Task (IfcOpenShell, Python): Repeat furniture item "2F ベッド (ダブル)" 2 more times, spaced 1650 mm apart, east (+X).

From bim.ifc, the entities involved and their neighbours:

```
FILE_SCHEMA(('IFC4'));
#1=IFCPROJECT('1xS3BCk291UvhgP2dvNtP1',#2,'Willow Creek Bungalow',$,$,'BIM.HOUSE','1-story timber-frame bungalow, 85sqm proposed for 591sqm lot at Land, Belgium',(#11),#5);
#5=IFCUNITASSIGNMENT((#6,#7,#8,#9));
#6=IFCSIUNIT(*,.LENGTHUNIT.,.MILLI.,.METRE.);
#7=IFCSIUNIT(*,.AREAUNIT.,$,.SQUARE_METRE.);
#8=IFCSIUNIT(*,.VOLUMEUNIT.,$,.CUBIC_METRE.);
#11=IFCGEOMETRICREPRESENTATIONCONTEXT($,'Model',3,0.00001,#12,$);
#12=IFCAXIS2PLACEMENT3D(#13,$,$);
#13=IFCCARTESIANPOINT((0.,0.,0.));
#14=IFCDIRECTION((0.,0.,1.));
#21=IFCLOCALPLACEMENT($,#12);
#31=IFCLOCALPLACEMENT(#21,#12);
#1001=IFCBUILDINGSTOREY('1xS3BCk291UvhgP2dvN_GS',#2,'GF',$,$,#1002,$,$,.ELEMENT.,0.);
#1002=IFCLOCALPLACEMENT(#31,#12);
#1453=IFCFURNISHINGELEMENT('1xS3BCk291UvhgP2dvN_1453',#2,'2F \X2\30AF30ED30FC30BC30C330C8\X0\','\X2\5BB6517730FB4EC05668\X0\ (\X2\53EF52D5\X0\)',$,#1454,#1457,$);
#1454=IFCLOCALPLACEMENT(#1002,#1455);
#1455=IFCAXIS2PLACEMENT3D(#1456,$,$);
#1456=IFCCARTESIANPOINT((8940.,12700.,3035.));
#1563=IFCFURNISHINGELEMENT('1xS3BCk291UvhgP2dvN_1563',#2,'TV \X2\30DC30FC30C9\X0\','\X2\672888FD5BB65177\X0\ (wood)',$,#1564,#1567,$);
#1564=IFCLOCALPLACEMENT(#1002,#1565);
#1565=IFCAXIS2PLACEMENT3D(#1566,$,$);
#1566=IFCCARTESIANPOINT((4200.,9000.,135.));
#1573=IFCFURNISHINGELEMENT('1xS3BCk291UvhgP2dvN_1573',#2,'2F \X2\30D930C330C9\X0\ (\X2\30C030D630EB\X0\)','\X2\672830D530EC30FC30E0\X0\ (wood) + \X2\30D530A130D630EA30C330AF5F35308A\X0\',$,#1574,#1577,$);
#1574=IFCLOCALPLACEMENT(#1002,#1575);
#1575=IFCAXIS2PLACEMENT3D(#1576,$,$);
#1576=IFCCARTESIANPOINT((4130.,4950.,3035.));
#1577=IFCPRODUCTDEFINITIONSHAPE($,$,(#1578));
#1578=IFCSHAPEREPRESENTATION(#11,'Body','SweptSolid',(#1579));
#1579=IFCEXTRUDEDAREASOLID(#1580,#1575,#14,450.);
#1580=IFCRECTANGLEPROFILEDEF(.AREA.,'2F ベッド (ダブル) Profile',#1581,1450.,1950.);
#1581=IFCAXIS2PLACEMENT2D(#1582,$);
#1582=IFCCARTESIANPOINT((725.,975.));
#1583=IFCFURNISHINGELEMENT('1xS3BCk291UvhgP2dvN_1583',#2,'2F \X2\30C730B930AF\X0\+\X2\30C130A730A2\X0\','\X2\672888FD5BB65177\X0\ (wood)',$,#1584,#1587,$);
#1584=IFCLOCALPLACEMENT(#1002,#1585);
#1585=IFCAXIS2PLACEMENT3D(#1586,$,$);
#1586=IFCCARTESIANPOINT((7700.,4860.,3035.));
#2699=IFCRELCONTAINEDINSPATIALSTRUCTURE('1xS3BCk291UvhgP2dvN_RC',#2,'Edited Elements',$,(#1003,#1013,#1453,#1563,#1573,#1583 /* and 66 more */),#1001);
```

```python
import numpy as np
import ifcopenshell
import ifcopenshell.api.geometry
import ifcopenshell.api.root
import ifcopenshell.util.element
import ifcopenshell.util.placement
import ifcopenshell.util.unit

model = ifcopenshell.open("bim.ifc")
unit_scale = ifcopenshell.util.unit.calculate_unit_scale(model)


def reuse_history(source, copy):
    """copy_class also copies each property set's owner history, people and application; keep the originals."""
    for rel in copy.IsDefinedBy:
        if rel.is_a("IfcRelDefinesByProperties") and (history := rel.RelatingPropertyDefinition.OwnerHistory):
            rel.RelatingPropertyDefinition.OwnerHistory = source.OwnerHistory
            ifcopenshell.util.element.remove_deep2(model, history)


source = model.by_guid("1xS3BCk291UvhgP2dvN_1573")
base = ifcopenshell.util.placement.get_local_placement(source.ObjectPlacement)
step = np.array([1.0, 0.0, 0.0]) * 1.65 / unit_scale

for i in range(1, 3):
    copy = ifcopenshell.api.root.copy_class(model, product=source)
    copy.Representation = ifcopenshell.util.element.copy_deep(
        model, source.Representation, exclude=["IfcGeometricRepresentationContext", "IfcRepresentationMap"]
    )
    reuse_history(source, copy)
    matrix = base.copy()
    matrix[:3, 3] += i * step
    print("added at", matrix[:3, 3].round(3) + 0.0)
    ifcopenshell.api.geometry.edit_object_placement(model, product=copy, matrix=matrix, is_si=False)

model.write("bim_rev.ifc")
```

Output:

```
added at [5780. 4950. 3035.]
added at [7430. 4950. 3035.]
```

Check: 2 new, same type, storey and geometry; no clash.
